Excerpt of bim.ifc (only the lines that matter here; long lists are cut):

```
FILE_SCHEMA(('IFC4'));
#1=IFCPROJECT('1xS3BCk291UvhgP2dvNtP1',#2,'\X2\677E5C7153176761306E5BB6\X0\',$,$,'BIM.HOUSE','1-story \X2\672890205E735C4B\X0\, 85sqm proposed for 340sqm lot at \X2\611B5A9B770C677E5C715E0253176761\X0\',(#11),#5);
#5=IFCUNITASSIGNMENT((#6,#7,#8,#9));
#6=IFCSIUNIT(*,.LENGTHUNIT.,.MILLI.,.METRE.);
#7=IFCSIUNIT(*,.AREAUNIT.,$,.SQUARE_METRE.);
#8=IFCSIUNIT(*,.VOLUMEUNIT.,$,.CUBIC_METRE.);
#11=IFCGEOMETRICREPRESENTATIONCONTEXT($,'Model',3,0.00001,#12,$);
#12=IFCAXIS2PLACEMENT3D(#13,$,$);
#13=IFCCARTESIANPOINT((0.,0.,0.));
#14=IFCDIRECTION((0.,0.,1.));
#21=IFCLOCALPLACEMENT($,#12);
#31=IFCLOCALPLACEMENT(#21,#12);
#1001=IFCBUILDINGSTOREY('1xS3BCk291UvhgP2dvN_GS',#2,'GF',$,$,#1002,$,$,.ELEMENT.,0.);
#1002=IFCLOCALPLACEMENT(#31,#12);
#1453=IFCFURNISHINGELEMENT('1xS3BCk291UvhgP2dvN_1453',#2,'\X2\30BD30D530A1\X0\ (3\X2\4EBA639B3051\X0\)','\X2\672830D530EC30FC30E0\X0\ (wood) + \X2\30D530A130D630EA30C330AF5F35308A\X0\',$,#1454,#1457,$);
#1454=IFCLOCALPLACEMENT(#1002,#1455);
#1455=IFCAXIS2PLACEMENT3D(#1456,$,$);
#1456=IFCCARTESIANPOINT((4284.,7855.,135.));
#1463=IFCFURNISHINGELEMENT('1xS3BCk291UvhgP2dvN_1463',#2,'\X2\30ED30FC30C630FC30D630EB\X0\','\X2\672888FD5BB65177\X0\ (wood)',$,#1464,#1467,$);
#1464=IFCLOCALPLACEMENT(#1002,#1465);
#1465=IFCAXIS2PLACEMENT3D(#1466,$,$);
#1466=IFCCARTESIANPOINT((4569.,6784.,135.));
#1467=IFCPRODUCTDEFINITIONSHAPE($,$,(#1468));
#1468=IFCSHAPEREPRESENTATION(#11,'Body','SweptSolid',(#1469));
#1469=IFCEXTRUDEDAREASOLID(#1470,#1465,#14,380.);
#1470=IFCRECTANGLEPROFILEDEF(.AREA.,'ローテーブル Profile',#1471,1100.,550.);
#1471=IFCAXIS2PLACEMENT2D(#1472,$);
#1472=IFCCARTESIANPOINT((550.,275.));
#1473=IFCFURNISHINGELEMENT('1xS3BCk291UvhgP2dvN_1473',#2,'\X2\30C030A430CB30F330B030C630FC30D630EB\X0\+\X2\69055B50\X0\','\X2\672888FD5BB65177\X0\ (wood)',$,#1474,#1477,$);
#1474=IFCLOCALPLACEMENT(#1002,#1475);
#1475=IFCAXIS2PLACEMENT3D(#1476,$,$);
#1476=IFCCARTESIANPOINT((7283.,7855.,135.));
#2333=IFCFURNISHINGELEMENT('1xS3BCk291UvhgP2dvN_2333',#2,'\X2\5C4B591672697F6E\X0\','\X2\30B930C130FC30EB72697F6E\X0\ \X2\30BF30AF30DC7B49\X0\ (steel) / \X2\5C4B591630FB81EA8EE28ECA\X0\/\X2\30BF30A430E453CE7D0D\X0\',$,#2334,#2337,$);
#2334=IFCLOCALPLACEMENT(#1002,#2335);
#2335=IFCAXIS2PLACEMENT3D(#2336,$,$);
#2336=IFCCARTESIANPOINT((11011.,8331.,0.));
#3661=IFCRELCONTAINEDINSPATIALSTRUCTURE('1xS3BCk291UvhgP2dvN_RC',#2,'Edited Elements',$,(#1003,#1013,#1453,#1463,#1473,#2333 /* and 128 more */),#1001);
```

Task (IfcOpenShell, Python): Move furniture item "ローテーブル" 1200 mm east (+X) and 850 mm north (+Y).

```python
import ifcopenshell
import ifcopenshell.api.geometry
import ifcopenshell.util.placement
import ifcopenshell.util.unit

model = ifcopenshell.open("bim.ifc")
unit_scale = ifcopenshell.util.unit.calculate_unit_scale(model)

item = model.by_guid("1xS3BCk291UvhgP2dvN_1463")
matrix = ifcopenshell.util.placement.get_local_placement(item.ObjectPlacement)
matrix[0, 3] += 1.2 / unit_scale
matrix[1, 3] += 0.85 / unit_scale
ifcopenshell.api.geometry.edit_object_placement(model, product=item, matrix=matrix, is_si=False)

print(ifcopenshell.util.placement.get_local_placement(item.ObjectPlacement).round(3) + 0.0)

model.write("bim_v2.ifc")
```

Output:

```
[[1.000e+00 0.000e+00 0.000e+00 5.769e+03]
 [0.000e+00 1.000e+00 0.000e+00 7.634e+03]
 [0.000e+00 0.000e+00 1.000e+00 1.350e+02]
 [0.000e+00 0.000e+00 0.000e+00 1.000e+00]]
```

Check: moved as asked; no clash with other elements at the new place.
